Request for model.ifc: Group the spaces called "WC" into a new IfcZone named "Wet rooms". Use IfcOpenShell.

First a look at what the model holds.

```python
import ifcopenshell

model = ifcopenshell.open("model.ifc")
print(model.schema)
seen = {}
for space in model.by_type("IfcSpace"):
    seen[space.LongName] = seen.get(space.LongName, 0) + 1
for name, count in sorted(seen.items(), key=str):
    print(count, "x", name)
print("zones:", [z.Name for z in model.by_type("IfcZone")][:20])
```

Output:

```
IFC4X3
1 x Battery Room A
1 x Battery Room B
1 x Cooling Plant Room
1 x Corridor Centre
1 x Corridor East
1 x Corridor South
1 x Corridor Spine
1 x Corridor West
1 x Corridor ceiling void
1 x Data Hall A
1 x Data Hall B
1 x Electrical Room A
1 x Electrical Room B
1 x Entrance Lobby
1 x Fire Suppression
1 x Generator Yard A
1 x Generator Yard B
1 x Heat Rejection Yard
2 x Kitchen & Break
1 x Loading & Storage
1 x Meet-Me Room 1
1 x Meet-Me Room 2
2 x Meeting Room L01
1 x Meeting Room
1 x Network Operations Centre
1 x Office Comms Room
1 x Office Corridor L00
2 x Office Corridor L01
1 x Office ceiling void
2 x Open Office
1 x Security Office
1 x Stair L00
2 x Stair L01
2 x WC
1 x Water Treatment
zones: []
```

```python
import ifcopenshell
import ifcopenshell.api.group
import ifcopenshell.api.root

model = ifcopenshell.open("model.ifc")

names = {"WC"}
spaces = [s for s in model.by_type("IfcSpace") if s.LongName in names]

zone = ifcopenshell.api.root.create_entity(model, ifc_class="IfcZone", name="Wet rooms")
ifcopenshell.api.group.assign_group(model, products=spaces, group=zone)
print(len(spaces), "spaces in", zone.Name)

model.write("model_rev.ifc")
```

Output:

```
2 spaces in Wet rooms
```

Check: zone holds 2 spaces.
